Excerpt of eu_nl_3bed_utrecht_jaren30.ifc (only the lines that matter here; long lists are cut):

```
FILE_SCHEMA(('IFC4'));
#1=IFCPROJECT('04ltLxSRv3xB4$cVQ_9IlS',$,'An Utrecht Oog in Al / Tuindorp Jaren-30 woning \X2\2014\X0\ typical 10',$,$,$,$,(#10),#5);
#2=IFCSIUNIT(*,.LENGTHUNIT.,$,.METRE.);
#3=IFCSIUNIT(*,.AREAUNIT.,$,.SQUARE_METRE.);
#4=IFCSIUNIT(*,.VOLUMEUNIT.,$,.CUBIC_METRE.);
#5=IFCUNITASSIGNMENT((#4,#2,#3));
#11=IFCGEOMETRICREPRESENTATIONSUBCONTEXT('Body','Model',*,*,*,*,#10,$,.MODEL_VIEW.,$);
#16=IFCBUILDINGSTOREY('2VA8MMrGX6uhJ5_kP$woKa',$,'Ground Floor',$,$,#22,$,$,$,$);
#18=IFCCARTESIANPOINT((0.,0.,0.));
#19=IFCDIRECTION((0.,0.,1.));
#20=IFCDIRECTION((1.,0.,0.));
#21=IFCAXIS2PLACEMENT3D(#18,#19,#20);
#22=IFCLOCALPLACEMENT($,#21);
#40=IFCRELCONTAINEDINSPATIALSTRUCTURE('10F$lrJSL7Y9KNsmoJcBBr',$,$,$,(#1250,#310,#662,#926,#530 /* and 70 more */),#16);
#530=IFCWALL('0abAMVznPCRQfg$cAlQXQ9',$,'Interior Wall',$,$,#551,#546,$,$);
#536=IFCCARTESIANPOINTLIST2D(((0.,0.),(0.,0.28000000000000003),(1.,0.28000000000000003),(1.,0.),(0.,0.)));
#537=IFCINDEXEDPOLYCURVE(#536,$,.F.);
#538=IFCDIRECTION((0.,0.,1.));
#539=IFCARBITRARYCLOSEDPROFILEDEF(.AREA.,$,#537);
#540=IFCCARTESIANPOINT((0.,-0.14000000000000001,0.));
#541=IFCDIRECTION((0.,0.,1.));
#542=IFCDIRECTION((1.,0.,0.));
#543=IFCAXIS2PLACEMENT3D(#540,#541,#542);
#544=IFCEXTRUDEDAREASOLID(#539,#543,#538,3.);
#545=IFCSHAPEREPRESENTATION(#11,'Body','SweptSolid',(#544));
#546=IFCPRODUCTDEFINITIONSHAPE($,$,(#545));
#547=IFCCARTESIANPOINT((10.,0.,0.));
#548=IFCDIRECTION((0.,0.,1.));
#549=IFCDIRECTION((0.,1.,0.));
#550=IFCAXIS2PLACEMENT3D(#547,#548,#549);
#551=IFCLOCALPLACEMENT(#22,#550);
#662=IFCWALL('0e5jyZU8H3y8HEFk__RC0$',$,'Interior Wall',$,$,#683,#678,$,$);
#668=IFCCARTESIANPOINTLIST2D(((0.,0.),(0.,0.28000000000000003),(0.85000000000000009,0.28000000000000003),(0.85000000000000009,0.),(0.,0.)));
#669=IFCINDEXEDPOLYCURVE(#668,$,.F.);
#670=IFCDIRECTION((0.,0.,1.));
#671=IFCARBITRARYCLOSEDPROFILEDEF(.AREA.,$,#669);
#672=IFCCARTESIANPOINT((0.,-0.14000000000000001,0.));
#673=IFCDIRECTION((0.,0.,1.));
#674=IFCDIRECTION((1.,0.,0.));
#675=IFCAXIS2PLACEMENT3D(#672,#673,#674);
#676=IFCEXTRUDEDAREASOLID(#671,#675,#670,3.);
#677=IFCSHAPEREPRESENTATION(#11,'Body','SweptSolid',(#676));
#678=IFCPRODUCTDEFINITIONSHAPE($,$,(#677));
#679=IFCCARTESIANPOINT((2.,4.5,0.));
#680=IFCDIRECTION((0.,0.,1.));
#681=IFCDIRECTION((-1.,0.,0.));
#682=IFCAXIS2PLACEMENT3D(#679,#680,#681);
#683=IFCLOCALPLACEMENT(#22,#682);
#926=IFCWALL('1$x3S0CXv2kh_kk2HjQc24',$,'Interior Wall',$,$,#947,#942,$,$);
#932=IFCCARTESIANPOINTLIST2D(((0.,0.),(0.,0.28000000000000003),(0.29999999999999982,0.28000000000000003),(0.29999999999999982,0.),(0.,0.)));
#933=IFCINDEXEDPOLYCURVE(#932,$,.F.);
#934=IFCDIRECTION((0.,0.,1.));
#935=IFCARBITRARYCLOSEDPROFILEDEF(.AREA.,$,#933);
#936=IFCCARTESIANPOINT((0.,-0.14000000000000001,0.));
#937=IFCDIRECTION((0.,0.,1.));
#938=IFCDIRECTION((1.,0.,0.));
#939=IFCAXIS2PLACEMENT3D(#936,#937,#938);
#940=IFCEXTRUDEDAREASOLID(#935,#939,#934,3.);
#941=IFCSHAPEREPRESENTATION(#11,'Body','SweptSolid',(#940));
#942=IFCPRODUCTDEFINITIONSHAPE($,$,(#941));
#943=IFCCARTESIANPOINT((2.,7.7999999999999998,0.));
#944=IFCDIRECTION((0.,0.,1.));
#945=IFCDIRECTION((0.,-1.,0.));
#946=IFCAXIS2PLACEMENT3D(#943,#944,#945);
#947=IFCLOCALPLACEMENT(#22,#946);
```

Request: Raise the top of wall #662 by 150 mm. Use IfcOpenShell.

```python
import ifcopenshell
import ifcopenshell.geom
import ifcopenshell.util.representation
import ifcopenshell.util.shape

model = ifcopenshell.open("eu_nl_3bed_utrecht_jaren30.ifc")
settings = ifcopenshell.geom.settings()


def volume(element):
    """Net volume in cubic metres, openings subtracted."""
    shape = ifcopenshell.geom.create_shape(settings, element)
    return ifcopenshell.util.shape.get_volume(shape.geometry)


wall = model.by_guid("0e5jyZU8H3y8HEFk__RC0$")
before = volume(wall)

body = ifcopenshell.util.representation.get_representation(wall, "Model", "Body")
solid = body.Items[0]
old_height = solid.Depth
solid.Depth += 0.15
after = volume(wall)

print(f"height {old_height:g} -> {solid.Depth:g}, volume {before:.3f} -> {after:.3f} m3")

model.write("eu_nl_3bed_utrecht_jaren30_updated.ifc")
```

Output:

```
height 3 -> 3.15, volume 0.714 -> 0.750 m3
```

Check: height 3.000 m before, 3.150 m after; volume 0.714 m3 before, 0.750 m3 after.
